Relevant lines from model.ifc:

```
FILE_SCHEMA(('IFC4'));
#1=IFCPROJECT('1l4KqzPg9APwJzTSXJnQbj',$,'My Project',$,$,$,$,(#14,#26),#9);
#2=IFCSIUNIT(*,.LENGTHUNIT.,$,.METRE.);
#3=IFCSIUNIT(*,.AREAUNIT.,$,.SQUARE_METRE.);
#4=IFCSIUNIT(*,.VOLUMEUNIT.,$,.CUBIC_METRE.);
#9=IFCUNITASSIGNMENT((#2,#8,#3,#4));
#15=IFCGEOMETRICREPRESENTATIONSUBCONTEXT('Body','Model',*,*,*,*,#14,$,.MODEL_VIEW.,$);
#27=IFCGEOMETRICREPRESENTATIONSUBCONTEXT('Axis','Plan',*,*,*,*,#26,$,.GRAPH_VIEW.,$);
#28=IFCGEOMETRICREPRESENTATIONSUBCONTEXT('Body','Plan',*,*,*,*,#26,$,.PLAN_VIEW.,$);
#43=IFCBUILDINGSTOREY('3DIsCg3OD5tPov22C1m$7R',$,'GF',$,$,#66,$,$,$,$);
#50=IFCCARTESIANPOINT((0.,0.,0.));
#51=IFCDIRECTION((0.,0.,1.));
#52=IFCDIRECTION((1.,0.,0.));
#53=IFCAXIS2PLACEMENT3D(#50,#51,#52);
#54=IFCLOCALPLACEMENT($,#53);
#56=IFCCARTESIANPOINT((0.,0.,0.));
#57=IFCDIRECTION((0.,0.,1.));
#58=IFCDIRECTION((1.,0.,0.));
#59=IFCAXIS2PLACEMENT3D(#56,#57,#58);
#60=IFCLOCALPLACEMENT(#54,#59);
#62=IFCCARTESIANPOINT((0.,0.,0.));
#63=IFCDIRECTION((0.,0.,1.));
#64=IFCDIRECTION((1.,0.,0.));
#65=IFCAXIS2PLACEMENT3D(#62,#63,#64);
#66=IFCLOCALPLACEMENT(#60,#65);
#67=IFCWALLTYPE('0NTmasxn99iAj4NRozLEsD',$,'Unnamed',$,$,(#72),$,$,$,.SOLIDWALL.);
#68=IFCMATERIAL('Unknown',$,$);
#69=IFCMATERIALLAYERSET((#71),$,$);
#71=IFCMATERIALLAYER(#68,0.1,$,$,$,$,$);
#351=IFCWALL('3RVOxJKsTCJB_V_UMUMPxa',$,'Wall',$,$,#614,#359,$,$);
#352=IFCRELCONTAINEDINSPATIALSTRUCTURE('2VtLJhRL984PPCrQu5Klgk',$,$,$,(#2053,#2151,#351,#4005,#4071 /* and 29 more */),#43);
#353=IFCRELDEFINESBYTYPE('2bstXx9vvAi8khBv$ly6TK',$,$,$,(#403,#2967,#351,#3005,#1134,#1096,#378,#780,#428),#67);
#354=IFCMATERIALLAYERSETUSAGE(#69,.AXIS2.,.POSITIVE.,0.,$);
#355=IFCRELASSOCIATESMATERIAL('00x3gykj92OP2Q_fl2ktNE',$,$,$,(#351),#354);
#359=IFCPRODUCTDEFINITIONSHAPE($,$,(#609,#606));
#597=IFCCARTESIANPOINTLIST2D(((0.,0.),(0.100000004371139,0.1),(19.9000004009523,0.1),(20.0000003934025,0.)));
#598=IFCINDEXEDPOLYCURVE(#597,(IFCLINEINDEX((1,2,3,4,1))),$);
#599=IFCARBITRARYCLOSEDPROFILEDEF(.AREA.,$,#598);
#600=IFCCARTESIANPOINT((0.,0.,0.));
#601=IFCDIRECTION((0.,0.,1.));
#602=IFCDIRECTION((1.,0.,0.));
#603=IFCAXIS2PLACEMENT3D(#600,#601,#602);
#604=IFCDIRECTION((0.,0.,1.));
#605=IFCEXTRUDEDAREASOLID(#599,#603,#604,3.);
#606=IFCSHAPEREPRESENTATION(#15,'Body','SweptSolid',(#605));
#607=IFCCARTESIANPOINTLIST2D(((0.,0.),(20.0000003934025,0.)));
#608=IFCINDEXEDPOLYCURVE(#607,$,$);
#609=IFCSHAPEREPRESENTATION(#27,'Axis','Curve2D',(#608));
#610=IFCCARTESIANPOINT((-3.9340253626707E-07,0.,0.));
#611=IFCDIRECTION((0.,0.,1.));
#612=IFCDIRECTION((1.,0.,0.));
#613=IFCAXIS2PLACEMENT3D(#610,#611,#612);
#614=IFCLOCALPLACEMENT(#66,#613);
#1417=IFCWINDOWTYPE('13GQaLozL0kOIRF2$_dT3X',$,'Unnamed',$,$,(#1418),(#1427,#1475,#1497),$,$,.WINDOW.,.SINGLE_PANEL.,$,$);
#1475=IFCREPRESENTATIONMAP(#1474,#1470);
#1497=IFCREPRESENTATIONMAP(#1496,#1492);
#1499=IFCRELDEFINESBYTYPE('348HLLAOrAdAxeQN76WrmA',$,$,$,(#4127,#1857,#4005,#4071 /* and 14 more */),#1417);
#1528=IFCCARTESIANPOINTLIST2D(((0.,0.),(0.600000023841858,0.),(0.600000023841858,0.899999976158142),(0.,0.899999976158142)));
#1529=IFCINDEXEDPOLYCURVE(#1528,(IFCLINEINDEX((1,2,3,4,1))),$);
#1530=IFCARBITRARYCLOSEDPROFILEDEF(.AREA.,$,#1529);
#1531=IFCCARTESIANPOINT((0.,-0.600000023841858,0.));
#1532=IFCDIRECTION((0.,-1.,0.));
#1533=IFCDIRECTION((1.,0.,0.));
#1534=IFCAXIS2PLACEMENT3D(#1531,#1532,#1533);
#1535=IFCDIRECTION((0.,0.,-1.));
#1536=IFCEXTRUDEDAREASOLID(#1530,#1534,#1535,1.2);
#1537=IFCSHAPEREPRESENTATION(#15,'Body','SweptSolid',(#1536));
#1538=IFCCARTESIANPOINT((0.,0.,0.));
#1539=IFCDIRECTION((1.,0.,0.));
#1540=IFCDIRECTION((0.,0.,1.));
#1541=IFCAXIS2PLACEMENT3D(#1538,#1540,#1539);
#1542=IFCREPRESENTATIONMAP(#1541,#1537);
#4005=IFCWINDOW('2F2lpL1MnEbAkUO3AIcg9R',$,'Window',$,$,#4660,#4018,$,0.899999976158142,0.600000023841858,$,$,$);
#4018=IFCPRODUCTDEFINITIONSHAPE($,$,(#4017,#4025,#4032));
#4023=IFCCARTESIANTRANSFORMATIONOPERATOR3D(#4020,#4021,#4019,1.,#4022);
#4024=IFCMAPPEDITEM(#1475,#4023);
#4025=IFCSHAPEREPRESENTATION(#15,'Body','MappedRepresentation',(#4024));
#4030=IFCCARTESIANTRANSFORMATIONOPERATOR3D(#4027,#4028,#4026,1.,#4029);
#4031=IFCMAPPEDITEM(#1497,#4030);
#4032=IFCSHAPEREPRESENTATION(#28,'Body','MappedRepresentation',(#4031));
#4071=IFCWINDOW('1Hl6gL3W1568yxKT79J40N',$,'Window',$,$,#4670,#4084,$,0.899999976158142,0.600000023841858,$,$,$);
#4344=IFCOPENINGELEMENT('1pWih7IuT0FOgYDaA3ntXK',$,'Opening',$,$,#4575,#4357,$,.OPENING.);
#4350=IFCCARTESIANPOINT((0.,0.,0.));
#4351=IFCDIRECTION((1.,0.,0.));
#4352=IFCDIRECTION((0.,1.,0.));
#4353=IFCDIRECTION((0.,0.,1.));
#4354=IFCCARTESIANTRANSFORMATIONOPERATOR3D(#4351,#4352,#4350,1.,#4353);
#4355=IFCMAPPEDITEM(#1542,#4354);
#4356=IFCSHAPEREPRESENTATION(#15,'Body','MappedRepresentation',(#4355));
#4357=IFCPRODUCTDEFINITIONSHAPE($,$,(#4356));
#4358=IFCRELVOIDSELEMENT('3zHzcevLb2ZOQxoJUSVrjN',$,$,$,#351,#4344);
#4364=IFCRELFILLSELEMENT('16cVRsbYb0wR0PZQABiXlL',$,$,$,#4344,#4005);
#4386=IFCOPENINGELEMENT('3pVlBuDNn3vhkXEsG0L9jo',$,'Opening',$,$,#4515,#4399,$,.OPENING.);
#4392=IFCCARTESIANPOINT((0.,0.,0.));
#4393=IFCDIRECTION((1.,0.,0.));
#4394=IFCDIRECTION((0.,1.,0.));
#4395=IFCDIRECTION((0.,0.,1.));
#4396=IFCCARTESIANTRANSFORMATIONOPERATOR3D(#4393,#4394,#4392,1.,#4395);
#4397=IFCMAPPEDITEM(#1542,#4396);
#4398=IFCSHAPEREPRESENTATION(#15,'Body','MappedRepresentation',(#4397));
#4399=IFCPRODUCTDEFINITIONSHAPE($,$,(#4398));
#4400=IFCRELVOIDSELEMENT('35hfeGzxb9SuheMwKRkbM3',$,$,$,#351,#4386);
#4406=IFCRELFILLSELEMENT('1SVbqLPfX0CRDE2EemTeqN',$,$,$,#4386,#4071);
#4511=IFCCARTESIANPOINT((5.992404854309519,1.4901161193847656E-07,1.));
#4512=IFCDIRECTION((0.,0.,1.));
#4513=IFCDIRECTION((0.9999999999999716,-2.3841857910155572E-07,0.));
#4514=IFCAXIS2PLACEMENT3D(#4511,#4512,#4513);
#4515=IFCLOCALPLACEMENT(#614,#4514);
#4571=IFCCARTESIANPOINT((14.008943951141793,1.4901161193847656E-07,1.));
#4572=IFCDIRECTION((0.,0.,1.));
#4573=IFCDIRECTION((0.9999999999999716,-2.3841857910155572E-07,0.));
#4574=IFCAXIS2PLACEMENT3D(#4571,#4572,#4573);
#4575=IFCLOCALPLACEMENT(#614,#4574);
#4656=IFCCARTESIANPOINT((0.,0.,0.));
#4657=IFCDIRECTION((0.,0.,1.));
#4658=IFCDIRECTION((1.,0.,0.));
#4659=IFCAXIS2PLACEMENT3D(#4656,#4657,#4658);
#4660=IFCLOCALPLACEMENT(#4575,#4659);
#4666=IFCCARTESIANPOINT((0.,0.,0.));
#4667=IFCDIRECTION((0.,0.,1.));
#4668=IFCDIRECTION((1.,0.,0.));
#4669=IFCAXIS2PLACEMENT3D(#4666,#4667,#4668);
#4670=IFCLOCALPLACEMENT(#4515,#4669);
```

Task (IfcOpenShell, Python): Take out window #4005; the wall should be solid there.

```python
import ifcopenshell
import ifcopenshell.api.feature
import ifcopenshell.api.root
import ifcopenshell.geom
import ifcopenshell.util.shape

model = ifcopenshell.open("model.ifc")
settings = ifcopenshell.geom.settings()


def volume(element):
    """Net volume in cubic metres, openings subtracted."""
    shape = ifcopenshell.geom.create_shape(settings, element)
    return ifcopenshell.util.shape.get_volume(shape.geometry)


window = model.by_guid("2F2lpL1MnEbAkUO3AIcg9R")
opening = window.FillsVoids[0].RelatingOpeningElement
wall = opening.VoidsElements[0].RelatingBuildingElement
before = volume(wall)

ifcopenshell.api.root.remove_product(model, product=window)
ifcopenshell.api.feature.remove_feature(model, feature=opening)

after = volume(wall)

print(f"wall volume {before:.3f} -> {after:.3f} m3")

model.write("model_updated.ifc")
```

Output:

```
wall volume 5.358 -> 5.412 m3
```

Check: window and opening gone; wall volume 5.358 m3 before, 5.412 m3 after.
